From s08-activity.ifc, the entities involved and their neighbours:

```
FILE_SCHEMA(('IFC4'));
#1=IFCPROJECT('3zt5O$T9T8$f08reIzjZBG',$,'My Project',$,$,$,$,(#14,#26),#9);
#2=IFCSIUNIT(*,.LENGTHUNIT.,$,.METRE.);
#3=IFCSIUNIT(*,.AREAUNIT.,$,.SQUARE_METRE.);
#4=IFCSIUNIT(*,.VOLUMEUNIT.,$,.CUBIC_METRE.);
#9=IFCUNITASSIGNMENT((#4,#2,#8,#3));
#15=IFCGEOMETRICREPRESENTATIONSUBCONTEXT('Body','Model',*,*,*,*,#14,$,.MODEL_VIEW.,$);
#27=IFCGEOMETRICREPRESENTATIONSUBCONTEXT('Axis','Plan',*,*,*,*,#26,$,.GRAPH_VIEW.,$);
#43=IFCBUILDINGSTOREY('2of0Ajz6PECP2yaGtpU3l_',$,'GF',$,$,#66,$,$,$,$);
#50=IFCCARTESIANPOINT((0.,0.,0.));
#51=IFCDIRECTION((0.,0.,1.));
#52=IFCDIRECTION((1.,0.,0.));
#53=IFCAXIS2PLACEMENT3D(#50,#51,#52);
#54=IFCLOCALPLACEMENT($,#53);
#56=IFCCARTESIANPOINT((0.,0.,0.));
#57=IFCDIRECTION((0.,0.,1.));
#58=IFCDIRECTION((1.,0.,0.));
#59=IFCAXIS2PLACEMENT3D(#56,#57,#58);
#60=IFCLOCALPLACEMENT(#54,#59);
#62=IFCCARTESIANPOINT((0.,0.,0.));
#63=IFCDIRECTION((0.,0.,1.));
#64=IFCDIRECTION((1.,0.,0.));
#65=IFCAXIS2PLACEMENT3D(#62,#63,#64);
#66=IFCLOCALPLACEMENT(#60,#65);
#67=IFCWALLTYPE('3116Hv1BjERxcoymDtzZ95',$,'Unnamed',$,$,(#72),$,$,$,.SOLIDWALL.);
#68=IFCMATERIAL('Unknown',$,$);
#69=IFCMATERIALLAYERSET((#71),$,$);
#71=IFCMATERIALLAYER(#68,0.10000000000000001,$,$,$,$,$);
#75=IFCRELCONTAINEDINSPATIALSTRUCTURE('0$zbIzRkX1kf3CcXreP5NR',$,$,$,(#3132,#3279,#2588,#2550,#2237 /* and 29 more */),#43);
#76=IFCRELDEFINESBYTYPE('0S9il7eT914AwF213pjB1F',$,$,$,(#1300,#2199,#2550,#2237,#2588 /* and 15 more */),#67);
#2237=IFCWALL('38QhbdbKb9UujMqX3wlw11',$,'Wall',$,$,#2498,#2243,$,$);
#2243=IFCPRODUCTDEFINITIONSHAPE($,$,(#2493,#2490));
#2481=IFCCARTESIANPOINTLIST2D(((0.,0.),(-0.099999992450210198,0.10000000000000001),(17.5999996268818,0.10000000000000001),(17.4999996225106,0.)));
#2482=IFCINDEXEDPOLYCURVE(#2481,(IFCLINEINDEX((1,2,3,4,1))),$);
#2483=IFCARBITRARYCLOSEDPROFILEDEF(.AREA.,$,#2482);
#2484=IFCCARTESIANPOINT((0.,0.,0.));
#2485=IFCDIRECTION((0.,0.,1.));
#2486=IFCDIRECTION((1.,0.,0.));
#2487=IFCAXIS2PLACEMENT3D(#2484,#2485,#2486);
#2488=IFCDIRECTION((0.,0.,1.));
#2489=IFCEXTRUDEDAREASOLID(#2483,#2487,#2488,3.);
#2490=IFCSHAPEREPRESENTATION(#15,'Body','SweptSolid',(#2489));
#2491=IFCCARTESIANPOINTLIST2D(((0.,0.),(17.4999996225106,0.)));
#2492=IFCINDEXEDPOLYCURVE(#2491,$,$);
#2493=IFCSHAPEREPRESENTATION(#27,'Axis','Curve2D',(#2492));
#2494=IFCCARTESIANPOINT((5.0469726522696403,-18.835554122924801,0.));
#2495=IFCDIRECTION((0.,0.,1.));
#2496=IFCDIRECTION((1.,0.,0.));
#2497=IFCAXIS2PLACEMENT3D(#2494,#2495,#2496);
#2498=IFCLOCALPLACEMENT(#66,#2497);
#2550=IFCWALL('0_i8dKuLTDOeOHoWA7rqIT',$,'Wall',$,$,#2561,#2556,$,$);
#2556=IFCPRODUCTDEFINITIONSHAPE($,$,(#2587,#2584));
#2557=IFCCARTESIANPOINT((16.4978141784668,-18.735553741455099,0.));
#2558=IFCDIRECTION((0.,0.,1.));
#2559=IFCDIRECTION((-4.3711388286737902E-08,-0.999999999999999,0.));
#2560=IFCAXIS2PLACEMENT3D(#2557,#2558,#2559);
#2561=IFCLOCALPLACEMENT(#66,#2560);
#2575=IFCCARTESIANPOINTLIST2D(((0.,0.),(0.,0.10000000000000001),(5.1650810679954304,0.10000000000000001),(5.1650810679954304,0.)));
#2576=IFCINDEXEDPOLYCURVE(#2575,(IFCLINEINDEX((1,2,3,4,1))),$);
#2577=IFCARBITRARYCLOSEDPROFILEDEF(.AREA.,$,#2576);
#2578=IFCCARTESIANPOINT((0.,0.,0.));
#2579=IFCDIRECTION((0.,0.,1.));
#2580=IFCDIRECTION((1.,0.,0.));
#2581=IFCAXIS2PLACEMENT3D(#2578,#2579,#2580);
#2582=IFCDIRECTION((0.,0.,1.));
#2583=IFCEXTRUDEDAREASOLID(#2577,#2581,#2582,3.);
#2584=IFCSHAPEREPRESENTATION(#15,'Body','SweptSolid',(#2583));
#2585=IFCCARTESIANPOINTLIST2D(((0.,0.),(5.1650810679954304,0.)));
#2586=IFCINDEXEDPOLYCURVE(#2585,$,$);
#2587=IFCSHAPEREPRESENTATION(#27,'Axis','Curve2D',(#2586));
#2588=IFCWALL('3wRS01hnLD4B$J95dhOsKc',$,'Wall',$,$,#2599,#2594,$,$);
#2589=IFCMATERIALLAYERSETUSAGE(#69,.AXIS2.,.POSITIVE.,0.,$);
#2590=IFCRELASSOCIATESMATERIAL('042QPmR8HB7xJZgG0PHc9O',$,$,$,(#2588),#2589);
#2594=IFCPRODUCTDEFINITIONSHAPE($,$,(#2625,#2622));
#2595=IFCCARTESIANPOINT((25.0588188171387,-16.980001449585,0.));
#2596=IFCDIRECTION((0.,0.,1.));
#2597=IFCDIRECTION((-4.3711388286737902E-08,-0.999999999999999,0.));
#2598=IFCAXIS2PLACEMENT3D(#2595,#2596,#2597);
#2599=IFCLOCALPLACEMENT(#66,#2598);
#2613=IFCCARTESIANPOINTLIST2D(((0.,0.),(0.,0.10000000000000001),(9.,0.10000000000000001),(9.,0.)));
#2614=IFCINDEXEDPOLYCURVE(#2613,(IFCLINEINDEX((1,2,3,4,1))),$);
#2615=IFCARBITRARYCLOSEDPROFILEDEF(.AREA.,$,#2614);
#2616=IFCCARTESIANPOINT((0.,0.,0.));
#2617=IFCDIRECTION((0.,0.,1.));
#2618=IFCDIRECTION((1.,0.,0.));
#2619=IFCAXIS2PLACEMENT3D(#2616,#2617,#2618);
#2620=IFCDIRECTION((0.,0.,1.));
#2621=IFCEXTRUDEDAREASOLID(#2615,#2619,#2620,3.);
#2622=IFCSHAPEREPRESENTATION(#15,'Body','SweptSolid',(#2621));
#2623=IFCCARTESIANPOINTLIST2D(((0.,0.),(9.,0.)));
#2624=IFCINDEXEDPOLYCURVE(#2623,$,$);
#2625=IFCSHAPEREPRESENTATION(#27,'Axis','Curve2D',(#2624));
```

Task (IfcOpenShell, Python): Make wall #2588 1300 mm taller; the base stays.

```python
import ifcopenshell
import ifcopenshell.geom
import ifcopenshell.util.representation
import ifcopenshell.util.shape
import ifcopenshell.util.unit

model = ifcopenshell.open("s08-activity.ifc")
unit_scale = ifcopenshell.util.unit.calculate_unit_scale(model)
settings = ifcopenshell.geom.settings()


def volume(element):
    """Net volume in cubic metres, openings subtracted."""
    shape = ifcopenshell.geom.create_shape(settings, element)
    return ifcopenshell.util.shape.get_volume(shape.geometry)


wall = model.by_guid("3wRS01hnLD4B$J95dhOsKc")
before = volume(wall)

body = ifcopenshell.util.representation.get_representation(wall, "Model", "Body")
solid = body.Items[0]
old_height = solid.Depth
solid.Depth += 1.3 / unit_scale
after = volume(wall)

print(f"height {old_height:g} -> {solid.Depth:g}, volume {before:.3f} -> {after:.3f} m3")

model.write("s08-activity-out.ifc")
```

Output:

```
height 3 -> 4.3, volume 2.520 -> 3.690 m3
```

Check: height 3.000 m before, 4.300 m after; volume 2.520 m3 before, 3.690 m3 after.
